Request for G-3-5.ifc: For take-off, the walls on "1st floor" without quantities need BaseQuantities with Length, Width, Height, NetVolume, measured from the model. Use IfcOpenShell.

First a look at what the model holds.

```python
import ifcopenshell
import ifcopenshell.util.element
import ifcopenshell.util.unit

model = ifcopenshell.open("G-3-5.ifc")
print(model.schema)
for unit_type in ("LENGTHUNIT", "AREAUNIT", "VOLUMEUNIT"):
    print(unit_type, ifcopenshell.util.unit.calculate_unit_scale(model, unit_type))
storey = next(s for s in model.by_type("IfcBuildingStorey") if s.Name == "1st floor")
walls = [e for e in ifcopenshell.util.element.get_decomposition(storey) if e.is_a("IfcWall")]
for e in sorted(walls, key=lambda e: e.id()):
    print(e.id(), e.is_a(), e.Name, list(ifcopenshell.util.element.get_psets(e, qtos_only=True)), sep=" | ")
```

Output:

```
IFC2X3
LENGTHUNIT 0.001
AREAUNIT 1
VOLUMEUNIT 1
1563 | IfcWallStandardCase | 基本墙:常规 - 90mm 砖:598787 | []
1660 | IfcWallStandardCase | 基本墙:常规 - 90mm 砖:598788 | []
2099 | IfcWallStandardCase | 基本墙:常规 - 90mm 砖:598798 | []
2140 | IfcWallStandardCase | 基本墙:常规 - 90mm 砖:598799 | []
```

```python
import ifcopenshell
import ifcopenshell.api.pset
import ifcopenshell.geom
import ifcopenshell.util.element
import ifcopenshell.util.shape
import ifcopenshell.util.unit

model = ifcopenshell.open("G-3-5.ifc")
unit_scale = ifcopenshell.util.unit.calculate_unit_scale(model)
volume_scale = ifcopenshell.util.unit.calculate_unit_scale(model, "VOLUMEUNIT")
settings = ifcopenshell.geom.settings()

storey = next(s for s in model.by_type("IfcBuildingStorey") if s.Name == "1st floor")
walls = [e for e in ifcopenshell.util.element.get_decomposition(storey) if e.is_a("IfcWall")]

for e in sorted(walls, key=lambda e: e.id()):
    if ifcopenshell.util.element.get_psets(e, qtos_only=True, should_inherit=False):
        continue
    # Geometry comes back in metres, in the element's own axes.
    shape = ifcopenshell.geom.create_shape(settings, e)
    values = {
        "Length": ifcopenshell.util.shape.get_x(shape.geometry) / unit_scale,
        "Width": ifcopenshell.util.shape.get_y(shape.geometry) / unit_scale,
        "Height": ifcopenshell.util.shape.get_z(shape.geometry) / unit_scale,
        "NetVolume": ifcopenshell.util.shape.get_volume(shape.geometry) / volume_scale,
    }
    qto = ifcopenshell.api.pset.add_qto(model, product=e, name="BaseQuantities")
    ifcopenshell.api.pset.edit_qto(model, qto=qto, properties=values)
    print(e.id(), {k: round(v, 3) for k, v in values.items()})

model.write("G-3-5_updated.ifc")
```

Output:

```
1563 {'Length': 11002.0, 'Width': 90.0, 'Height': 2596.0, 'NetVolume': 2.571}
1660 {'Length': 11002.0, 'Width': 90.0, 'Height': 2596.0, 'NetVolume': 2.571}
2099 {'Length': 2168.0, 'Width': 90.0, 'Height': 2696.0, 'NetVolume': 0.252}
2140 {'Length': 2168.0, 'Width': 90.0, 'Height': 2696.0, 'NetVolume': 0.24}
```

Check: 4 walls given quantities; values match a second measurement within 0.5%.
